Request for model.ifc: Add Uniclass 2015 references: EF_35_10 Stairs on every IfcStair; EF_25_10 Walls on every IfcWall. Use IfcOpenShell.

First a look at what the model holds.

```python
import ifcopenshell

model = ifcopenshell.open("model.ifc")
print(model.schema)
print("classifications:", [c.Name for c in model.by_type("IfcClassification")])
for ifc_class in ("IfcDoor", "IfcRoof", "IfcStair", "IfcWall", "IfcWindow"):
    print(ifc_class, len(model.by_type(ifc_class)))
```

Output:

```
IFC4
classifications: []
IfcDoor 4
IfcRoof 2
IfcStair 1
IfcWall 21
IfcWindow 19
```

```python
import ifcopenshell
import ifcopenshell.api.classification

model = ifcopenshell.open("model.ifc")

system = ifcopenshell.api.classification.add_classification(model, classification="Uniclass 2015")

codes = {
    "IfcStair": ("EF_35_10", "Stairs"),
    "IfcWall": ("EF_25_10", "Walls"),
}
for ifc_class, (code, name) in codes.items():
    products = model.by_type(ifc_class)
    ifcopenshell.api.classification.add_reference(
        model, products=products, classification=system, identification=code, name=name
    )
    print(code, len(products))

model.write("model_rev.ifc")
```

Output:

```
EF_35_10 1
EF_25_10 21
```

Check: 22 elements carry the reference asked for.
